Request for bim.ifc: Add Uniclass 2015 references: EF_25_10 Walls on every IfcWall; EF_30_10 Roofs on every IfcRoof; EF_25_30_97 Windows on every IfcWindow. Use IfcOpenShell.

First a look at what the model holds.

```python
import ifcopenshell

model = ifcopenshell.open("bim.ifc")
print(model.schema)
print("classifications:", [c.Name for c in model.by_type("IfcClassification")])
for ifc_class in ("IfcDoor", "IfcRoof", "IfcStair", "IfcWall", "IfcWindow"):
    print(ifc_class, len(model.by_type(ifc_class)))
```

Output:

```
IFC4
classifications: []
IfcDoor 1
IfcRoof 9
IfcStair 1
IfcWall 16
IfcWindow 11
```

```python
import ifcopenshell
import ifcopenshell.api.classification

model = ifcopenshell.open("bim.ifc")

system = ifcopenshell.api.classification.add_classification(model, classification="Uniclass 2015")

codes = {
    "IfcWall": ("EF_25_10", "Walls"),
    "IfcRoof": ("EF_30_10", "Roofs"),
    "IfcWindow": ("EF_25_30_97", "Windows"),
}
for ifc_class, (code, name) in codes.items():
    products = model.by_type(ifc_class)
    ifcopenshell.api.classification.add_reference(
        model, products=products, classification=system, identification=code, name=name
    )
    print(code, len(products))

model.write("bim_rev.ifc")
```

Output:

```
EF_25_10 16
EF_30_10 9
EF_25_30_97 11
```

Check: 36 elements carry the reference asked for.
